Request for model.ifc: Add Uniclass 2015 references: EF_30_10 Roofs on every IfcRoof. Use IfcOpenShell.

First a look at what the model holds.

```python
import ifcopenshell

model = ifcopenshell.open("model.ifc")
print(model.schema)
print("classifications:", [c.Name for c in model.by_type("IfcClassification")])
for ifc_class in ("IfcDoor", "IfcRoof", "IfcStair", "IfcWall", "IfcWindow"):
    print(ifc_class, len(model.by_type(ifc_class)))
```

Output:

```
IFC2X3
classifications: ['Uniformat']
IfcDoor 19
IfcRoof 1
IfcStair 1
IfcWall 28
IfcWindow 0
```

```python
import ifcopenshell
import ifcopenshell.api.classification

model = ifcopenshell.open("model.ifc")

# IFC2X3 requires Source and Edition and has no link from the project to the system.
system = model.create_entity("IfcClassification", Source="NBS", Edition="2015", Name="Uniclass 2015")

codes = {
    "IfcRoof": ("EF_30_10", "Roofs"),
}
for ifc_class, (code, name) in codes.items():
    products = model.by_type(ifc_class)
    ifcopenshell.api.classification.add_reference(
        model, products=products, classification=system, identification=code, name=name
    )
    print(code, len(products))

model.write("model_rev.ifc")
```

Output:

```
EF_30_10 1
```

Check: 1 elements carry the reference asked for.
